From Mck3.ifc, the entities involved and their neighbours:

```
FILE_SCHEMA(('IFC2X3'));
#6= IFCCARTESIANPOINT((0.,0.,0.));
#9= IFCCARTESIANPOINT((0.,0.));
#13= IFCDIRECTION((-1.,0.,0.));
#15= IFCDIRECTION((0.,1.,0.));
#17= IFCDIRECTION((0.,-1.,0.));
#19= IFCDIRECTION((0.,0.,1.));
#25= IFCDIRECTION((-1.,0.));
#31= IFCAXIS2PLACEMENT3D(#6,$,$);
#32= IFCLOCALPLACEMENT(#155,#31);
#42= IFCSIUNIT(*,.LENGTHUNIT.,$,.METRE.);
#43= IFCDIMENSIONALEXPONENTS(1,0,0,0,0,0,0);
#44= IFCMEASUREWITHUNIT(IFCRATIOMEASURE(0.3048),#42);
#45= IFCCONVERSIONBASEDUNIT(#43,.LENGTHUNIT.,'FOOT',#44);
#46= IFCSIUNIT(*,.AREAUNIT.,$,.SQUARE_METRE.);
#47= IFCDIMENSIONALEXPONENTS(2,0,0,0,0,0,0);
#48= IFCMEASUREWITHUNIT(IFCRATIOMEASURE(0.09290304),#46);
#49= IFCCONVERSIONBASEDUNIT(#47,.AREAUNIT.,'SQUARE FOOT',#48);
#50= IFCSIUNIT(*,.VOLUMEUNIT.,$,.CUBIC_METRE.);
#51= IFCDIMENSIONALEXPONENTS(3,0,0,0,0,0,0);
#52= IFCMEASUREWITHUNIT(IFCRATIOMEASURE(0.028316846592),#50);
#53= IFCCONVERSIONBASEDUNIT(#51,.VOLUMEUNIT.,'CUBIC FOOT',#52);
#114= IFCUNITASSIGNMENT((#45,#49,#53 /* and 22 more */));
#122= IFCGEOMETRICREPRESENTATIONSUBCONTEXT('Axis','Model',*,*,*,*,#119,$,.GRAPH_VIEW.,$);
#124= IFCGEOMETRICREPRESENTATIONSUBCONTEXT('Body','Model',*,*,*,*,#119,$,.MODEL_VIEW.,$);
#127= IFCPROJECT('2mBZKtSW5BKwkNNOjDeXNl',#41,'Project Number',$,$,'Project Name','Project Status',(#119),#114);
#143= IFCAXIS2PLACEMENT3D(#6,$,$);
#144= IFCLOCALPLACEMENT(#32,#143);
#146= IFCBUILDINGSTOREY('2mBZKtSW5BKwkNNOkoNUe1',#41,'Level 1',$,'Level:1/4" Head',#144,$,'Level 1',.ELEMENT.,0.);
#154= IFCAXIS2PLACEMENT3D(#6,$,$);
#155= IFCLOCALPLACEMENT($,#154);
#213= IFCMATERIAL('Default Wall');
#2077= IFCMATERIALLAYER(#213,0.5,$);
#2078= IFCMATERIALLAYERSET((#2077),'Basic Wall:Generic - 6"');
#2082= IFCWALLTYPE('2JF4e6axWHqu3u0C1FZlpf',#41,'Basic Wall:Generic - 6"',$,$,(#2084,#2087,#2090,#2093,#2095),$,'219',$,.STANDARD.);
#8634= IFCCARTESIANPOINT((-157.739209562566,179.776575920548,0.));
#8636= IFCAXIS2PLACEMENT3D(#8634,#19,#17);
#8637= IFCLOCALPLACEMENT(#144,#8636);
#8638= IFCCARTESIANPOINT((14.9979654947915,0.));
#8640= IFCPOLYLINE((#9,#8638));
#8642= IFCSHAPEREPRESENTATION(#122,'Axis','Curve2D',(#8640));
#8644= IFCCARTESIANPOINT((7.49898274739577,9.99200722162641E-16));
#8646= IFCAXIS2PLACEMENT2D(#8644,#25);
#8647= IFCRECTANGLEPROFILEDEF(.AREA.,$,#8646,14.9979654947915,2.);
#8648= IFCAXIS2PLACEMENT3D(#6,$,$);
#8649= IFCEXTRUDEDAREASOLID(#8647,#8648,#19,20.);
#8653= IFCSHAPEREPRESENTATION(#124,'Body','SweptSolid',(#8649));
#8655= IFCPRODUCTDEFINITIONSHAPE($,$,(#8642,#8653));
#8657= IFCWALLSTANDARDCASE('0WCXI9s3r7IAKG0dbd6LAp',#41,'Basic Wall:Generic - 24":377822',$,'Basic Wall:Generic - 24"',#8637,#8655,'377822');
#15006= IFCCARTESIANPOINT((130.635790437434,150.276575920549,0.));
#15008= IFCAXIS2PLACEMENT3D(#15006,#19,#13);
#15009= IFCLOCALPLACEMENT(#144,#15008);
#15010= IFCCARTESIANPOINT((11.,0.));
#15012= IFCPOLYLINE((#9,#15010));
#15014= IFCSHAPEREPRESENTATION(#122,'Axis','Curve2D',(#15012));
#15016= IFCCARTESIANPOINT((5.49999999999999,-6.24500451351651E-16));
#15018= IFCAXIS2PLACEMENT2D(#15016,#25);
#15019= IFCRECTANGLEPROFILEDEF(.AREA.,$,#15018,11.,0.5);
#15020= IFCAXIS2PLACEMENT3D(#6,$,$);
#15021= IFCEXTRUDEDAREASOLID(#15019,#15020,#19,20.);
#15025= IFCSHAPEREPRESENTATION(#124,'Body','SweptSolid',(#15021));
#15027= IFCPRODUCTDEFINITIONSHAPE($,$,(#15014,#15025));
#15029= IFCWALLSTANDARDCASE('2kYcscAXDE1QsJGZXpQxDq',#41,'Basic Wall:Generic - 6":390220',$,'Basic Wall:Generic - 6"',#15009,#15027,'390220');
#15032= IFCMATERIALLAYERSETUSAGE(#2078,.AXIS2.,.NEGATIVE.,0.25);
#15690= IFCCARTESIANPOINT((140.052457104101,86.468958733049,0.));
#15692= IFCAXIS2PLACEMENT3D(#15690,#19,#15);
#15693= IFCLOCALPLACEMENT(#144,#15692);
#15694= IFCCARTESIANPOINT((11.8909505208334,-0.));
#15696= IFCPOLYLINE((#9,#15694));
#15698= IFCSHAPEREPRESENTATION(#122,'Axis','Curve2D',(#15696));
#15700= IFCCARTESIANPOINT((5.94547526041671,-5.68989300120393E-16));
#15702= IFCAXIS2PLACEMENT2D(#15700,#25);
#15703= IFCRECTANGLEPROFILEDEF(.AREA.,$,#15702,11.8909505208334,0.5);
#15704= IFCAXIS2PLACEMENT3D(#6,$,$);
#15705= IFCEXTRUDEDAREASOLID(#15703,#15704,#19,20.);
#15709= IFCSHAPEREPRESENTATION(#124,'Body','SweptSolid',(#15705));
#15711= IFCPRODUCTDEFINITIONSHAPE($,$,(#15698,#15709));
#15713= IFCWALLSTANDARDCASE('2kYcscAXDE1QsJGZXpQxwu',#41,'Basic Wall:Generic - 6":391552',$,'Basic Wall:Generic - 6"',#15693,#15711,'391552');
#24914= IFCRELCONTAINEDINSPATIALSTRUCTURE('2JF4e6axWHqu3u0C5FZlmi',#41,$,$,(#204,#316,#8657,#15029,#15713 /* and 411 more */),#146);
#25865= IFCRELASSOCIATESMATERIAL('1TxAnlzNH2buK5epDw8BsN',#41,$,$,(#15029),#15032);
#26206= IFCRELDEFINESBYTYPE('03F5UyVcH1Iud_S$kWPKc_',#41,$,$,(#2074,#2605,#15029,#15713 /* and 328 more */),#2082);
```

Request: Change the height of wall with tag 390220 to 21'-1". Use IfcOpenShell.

```python
import ifcopenshell
import ifcopenshell.geom
import ifcopenshell.util.representation
import ifcopenshell.util.shape
import ifcopenshell.util.unit

model = ifcopenshell.open("Mck3.ifc")
unit_scale = ifcopenshell.util.unit.calculate_unit_scale(model)
settings = ifcopenshell.geom.settings()


def volume(element):
    """Net volume in cubic metres, openings subtracted."""
    shape = ifcopenshell.geom.create_shape(settings, element)
    return ifcopenshell.util.shape.get_volume(shape.geometry)


wall = model.by_guid("2kYcscAXDE1QsJGZXpQxDq")
before = volume(wall)

body = ifcopenshell.util.representation.get_representation(wall, "Model", "Body")
solid = body.Items[0]
old_height = solid.Depth
solid.Depth = 253 * 0.0254 / unit_scale
after = volume(wall)

print(f"height {old_height:g} -> {solid.Depth:g}, volume {before:.3f} -> {after:.3f} m3")

model.write("Mck3_v2.ifc")
```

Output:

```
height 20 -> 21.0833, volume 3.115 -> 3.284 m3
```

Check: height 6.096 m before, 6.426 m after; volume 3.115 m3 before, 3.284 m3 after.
